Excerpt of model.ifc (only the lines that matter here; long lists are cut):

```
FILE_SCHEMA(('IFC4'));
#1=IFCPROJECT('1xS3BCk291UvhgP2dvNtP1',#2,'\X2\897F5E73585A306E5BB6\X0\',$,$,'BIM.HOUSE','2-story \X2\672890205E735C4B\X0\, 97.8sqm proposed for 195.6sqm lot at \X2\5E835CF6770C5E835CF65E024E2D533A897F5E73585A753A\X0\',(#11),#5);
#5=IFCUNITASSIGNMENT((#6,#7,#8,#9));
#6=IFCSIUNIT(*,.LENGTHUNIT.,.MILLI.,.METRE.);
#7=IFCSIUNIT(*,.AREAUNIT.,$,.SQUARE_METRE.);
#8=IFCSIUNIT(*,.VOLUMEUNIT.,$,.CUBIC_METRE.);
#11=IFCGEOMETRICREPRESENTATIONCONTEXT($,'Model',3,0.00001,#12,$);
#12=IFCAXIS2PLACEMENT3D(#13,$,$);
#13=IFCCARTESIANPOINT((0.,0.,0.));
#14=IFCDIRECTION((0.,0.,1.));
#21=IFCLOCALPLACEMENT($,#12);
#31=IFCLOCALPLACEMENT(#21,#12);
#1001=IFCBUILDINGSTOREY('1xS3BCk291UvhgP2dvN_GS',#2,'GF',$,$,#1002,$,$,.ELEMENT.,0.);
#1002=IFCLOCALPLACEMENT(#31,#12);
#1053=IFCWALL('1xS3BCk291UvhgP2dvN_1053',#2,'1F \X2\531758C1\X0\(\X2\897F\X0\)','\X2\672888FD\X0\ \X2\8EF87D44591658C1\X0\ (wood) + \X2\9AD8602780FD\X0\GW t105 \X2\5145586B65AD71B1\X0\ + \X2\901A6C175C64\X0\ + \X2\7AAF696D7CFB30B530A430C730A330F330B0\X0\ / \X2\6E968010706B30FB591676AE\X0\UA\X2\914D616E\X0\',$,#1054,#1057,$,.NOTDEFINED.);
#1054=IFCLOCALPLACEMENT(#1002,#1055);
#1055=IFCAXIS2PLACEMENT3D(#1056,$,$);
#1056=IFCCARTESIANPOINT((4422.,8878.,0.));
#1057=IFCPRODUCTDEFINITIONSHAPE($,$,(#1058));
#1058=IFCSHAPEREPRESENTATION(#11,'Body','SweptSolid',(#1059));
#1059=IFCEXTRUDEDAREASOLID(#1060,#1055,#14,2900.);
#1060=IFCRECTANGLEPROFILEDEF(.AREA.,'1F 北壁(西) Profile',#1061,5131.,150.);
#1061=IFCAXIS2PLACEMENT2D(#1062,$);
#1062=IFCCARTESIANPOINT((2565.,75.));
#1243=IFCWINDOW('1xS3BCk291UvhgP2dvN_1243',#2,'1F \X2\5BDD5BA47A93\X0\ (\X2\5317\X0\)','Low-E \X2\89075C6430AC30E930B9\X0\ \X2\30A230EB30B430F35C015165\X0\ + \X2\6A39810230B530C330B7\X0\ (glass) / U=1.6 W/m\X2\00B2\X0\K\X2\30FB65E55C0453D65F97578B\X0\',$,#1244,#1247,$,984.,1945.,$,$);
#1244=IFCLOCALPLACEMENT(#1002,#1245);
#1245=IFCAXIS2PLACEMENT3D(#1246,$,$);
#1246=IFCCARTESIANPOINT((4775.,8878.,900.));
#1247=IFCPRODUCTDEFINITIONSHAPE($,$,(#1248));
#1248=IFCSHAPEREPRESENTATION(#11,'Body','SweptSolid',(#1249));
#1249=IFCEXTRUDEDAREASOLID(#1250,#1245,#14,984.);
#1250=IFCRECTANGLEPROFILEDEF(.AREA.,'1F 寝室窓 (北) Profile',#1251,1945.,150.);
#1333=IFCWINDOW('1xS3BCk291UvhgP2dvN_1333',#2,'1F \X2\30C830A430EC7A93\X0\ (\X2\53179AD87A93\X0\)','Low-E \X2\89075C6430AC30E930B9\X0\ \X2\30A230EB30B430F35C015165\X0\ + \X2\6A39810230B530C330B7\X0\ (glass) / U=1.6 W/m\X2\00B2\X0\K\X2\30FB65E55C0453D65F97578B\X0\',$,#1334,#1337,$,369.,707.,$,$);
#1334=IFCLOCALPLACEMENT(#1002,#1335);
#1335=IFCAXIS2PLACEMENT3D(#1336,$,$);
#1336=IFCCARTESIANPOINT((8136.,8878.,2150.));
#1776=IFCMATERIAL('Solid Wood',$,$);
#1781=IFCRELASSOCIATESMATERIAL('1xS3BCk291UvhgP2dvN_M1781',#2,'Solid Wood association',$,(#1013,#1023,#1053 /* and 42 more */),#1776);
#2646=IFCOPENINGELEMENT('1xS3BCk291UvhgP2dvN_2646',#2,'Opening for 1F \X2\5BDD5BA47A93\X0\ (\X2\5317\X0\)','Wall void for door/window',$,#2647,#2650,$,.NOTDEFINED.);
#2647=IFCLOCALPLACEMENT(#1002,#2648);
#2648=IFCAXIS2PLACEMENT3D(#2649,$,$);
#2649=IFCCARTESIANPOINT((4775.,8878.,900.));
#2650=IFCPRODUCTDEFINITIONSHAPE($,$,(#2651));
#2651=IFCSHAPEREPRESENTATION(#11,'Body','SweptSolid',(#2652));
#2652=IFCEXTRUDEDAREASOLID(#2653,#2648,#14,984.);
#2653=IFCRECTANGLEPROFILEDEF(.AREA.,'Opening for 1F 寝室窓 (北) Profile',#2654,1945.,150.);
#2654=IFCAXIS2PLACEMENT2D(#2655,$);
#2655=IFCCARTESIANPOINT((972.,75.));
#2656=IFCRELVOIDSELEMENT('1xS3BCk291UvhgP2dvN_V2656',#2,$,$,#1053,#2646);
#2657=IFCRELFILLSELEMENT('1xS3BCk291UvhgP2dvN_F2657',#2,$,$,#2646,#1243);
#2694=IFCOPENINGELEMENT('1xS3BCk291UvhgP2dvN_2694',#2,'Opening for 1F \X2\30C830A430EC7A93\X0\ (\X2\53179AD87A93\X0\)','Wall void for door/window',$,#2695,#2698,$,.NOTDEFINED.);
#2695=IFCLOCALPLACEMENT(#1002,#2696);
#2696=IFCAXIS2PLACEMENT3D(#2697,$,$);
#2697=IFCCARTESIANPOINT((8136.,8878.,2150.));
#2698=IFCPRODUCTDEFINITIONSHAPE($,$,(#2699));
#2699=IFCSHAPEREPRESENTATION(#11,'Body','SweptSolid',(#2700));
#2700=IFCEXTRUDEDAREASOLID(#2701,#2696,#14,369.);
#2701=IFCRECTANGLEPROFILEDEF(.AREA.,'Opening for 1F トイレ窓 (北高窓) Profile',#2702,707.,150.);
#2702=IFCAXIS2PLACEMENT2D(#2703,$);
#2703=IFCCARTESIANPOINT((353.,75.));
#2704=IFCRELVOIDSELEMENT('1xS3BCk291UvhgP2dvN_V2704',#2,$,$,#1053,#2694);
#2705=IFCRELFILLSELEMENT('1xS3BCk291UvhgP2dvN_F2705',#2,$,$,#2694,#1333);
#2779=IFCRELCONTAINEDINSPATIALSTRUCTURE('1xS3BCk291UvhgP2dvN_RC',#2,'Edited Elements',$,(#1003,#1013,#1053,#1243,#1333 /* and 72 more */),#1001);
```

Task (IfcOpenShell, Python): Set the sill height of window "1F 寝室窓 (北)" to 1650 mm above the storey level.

```python
import numpy as np
import ifcopenshell
import ifcopenshell.api.geometry
import ifcopenshell.geom
import ifcopenshell.util.element
import ifcopenshell.util.placement
import ifcopenshell.util.shape
import ifcopenshell.util.unit

model = ifcopenshell.open("model.ifc")
unit_scale = ifcopenshell.util.unit.calculate_unit_scale(model)

window = model.by_guid("1xS3BCk291UvhgP2dvN_1243")
opening = window.FillsVoids[0].RelatingOpeningElement
storey = ifcopenshell.util.element.get_container(window, ifc_class="IfcBuildingStorey")
level = ifcopenshell.util.placement.get_local_placement(storey.ObjectPlacement)[2, 3]

# The opening's origin need not be at the sill, so measure its lowest point.
shape = ifcopenshell.geom.create_shape(ifcopenshell.geom.settings(), opening)
bottom = ifcopenshell.util.shape.get_shape_bottom_elevation(shape, shape.geometry) / unit_scale
dz = level + 1.65 / unit_scale - bottom

shift = np.array([0.0, 0.0, dz])
# The window is not placed relative to its opening, so move both.
for product in (opening, window):
    matrix = ifcopenshell.util.placement.get_local_placement(product.ObjectPlacement)
    matrix[:3, 3] += shift
    ifcopenshell.api.geometry.edit_object_placement(model, product=product, matrix=matrix, is_si=False)

print(f"moved by {dz * unit_scale:+.3f} m")

model.write("model_updated.ifc")
```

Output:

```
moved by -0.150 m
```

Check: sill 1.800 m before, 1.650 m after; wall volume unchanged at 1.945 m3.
